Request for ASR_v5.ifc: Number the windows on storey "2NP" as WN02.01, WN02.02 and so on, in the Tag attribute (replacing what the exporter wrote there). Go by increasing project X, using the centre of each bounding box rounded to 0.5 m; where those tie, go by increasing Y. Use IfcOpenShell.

First a look at what the model holds.

```python
import ifcopenshell
import ifcopenshell.util.element
import ifcopenshell.util.placement

model = ifcopenshell.open("ASR_v5.ifc")
print(model.schema)
storey = next(s for s in model.by_type("IfcBuildingStorey") if s.Name == "2NP")
windows = [e for e in ifcopenshell.util.element.get_decomposition(storey) if e.is_a("IfcWindow")]
for e in sorted(windows, key=lambda e: e.id()):
    origin = ifcopenshell.util.placement.get_local_placement(e.ObjectPlacement)[:3, 3]
    print(e.id(), e.Tag, e.Name, origin.round(2) + 0.0, sep=" | ")
```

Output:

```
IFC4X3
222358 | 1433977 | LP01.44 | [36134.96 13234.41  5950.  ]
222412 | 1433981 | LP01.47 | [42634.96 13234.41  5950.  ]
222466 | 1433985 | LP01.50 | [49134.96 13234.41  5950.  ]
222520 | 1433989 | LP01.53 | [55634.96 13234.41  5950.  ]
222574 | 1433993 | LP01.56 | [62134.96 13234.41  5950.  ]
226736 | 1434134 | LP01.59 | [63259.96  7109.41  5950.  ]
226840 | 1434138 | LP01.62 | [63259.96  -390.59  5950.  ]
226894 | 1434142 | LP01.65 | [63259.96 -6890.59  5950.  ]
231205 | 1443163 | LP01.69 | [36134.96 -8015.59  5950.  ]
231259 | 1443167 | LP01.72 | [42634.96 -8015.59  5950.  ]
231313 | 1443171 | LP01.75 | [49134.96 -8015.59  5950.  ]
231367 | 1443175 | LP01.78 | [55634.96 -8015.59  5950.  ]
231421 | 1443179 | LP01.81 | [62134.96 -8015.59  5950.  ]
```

```python
import ifcopenshell
import ifcopenshell.geom
import ifcopenshell.util.element
import ifcopenshell.util.shape

model = ifcopenshell.open("ASR_v5.ifc")
settings = ifcopenshell.geom.settings()
settings.set("use-world-coords", True)


def centre(element):
    shape = ifcopenshell.geom.create_shape(settings, element)
    return ifcopenshell.util.shape.get_bbox_centroid(shape.geometry)


storey = next(s for s in model.by_type("IfcBuildingStorey") if s.Name == "2NP")
windows = [e for e in ifcopenshell.util.element.get_decomposition(storey) if e.is_a("IfcWindow")]

# Insertion points can sit at a corner or the storey origin, so sort by the geometry (in metres).
centres = {e: centre(e) for e in windows}
windows.sort(key=lambda e: (round(centres[e][0] / 0.5), centres[e][1]))

for i, e in enumerate(windows, start=1):
    number = f"WN02.{i:02d}"
    e.Tag = number
    print(e.id(), number)

model.write("ASR_v5_rev.ifc")
```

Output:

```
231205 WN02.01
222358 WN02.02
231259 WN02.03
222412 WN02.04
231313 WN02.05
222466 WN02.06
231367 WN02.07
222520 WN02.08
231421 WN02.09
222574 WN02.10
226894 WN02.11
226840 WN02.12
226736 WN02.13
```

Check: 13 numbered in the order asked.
